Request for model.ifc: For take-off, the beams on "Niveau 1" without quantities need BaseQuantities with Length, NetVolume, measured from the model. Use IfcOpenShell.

First a look at what the model holds.

```python
import ifcopenshell
import ifcopenshell.util.element
import ifcopenshell.util.unit

model = ifcopenshell.open("model.ifc")
print(model.schema)
for unit_type in ("LENGTHUNIT", "AREAUNIT", "VOLUMEUNIT"):
    print(unit_type, ifcopenshell.util.unit.calculate_unit_scale(model, unit_type))
storey = next(s for s in model.by_type("IfcBuildingStorey") if s.Name == "Niveau 1")
beams = [e for e in ifcopenshell.util.element.get_decomposition(storey) if e.is_a("IfcBeam")]
for e in sorted(beams, key=lambda e: e.id()):
    print(e.id(), e.is_a(), e.Name, list(ifcopenshell.util.element.get_psets(e, qtos_only=True)), sep=" | ")
```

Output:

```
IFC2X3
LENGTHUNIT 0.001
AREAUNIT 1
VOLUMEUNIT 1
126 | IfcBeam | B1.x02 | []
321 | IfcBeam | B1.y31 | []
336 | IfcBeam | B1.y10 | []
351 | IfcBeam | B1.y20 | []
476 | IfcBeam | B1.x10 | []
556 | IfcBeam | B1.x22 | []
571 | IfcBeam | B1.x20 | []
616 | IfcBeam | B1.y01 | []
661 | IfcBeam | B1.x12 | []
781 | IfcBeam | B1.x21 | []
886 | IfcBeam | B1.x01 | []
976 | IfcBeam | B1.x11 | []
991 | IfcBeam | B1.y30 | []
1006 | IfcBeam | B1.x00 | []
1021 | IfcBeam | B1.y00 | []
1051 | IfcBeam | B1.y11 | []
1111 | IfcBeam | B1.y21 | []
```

```python
import ifcopenshell
import ifcopenshell.api.pset
import ifcopenshell.geom
import ifcopenshell.util.element
import ifcopenshell.util.shape
import ifcopenshell.util.unit

model = ifcopenshell.open("model.ifc")
unit_scale = ifcopenshell.util.unit.calculate_unit_scale(model)
volume_scale = ifcopenshell.util.unit.calculate_unit_scale(model, "VOLUMEUNIT")
settings = ifcopenshell.geom.settings()

storey = next(s for s in model.by_type("IfcBuildingStorey") if s.Name == "Niveau 1")
beams = [e for e in ifcopenshell.util.element.get_decomposition(storey) if e.is_a("IfcBeam")]

for e in sorted(beams, key=lambda e: e.id()):
    if ifcopenshell.util.element.get_psets(e, qtos_only=True, should_inherit=False):
        continue
    # Geometry comes back in metres, in the element's own axes.
    shape = ifcopenshell.geom.create_shape(settings, e)
    values = {
        "Length": ifcopenshell.util.shape.get_max_xyz(shape.geometry) / unit_scale,
        "NetVolume": ifcopenshell.util.shape.get_volume(shape.geometry) / volume_scale,
    }
    qto = ifcopenshell.api.pset.add_qto(model, product=e, name="BaseQuantities")
    ifcopenshell.api.pset.edit_qto(model, qto=qto, properties=values)
    print(e.id(), {k: round(v, 3) for k, v in values.items()})

model.write("model_v2.ifc")
```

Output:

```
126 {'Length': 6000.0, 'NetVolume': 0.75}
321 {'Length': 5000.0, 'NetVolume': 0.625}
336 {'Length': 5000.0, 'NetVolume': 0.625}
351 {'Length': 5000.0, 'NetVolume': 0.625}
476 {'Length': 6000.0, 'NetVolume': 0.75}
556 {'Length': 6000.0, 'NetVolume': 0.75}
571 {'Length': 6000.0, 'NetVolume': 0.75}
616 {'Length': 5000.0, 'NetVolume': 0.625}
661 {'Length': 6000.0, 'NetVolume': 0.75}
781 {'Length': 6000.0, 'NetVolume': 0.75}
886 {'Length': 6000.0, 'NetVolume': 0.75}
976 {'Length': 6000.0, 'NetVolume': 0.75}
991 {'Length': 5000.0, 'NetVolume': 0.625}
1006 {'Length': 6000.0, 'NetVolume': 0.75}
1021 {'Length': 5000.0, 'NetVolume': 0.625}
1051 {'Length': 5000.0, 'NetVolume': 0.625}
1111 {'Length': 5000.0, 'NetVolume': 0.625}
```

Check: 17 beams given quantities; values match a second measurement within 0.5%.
